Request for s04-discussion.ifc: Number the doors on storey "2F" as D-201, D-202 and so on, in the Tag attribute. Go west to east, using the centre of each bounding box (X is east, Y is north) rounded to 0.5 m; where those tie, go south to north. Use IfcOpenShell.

First a look at what the model holds.

```python
import ifcopenshell
import ifcopenshell.util.element
import ifcopenshell.util.placement

model = ifcopenshell.open("s04-discussion.ifc")
print(model.schema)
storey = next(s for s in model.by_type("IfcBuildingStorey") if s.Name == "2F")
doors = [e for e in ifcopenshell.util.element.get_decomposition(storey) if e.is_a("IfcDoor")]
for e in sorted(doors, key=lambda e: e.id()):
    origin = ifcopenshell.util.placement.get_local_placement(e.ObjectPlacement)[:3, 3]
    print(e.id(), e.Tag, e.Name, origin.round(2) + 0.0, sep=" | ")
```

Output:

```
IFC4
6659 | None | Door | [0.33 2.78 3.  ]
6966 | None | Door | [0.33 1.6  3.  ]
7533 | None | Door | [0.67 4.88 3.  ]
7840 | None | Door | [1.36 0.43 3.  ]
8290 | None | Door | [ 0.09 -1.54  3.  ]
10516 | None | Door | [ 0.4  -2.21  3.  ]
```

```python
import ifcopenshell
import ifcopenshell.geom
import ifcopenshell.util.element
import ifcopenshell.util.shape

model = ifcopenshell.open("s04-discussion.ifc")
settings = ifcopenshell.geom.settings()
settings.set("use-world-coords", True)


def centre(element):
    shape = ifcopenshell.geom.create_shape(settings, element)
    return ifcopenshell.util.shape.get_bbox_centroid(shape.geometry)


storey = next(s for s in model.by_type("IfcBuildingStorey") if s.Name == "2F")
doors = [e for e in ifcopenshell.util.element.get_decomposition(storey) if e.is_a("IfcDoor")]

# Insertion points can sit at a corner or the storey origin, so sort by the geometry (in metres).
centres = {e: centre(e) for e in doors}
doors.sort(key=lambda e: (round(centres[e][0] / 0.5), centres[e][1]))

for i, e in enumerate(doors, start=1):
    number = f"D-2{i:02d}"
    e.Tag = number
    print(e.id(), number)

model.write("s04-discussion_rev.ifc")
```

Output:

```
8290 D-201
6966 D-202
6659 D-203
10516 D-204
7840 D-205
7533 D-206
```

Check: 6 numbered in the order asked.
